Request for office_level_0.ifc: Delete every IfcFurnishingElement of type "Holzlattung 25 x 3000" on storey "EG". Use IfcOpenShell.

First a look at what the model holds.

```python
import ifcopenshell
import ifcopenshell.util.element

model = ifcopenshell.open("office_level_0.ifc")
print(model.schema)
storey = next(s for s in model.by_type("IfcBuildingStorey") if s.Name == "EG")
furniture = [e for e in ifcopenshell.util.element.get_decomposition(storey) if e.is_a("IfcFurnishingElement")]
seen = {}
for e in furniture:
    element_type = ifcopenshell.util.element.get_type(e)
    name = element_type.Name if element_type not in (None, e) else None
    seen[name] = seen.get(name, 0) + 1
for name, count in sorted(seen.items(), key=str):
    print(count, "x", name)
```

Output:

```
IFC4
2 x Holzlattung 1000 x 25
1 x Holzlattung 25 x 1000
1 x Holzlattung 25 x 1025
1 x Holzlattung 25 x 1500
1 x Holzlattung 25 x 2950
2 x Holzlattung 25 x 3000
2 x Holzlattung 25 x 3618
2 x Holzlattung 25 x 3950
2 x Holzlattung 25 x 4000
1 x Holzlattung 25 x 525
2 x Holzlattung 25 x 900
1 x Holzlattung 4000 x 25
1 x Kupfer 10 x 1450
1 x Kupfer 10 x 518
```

```python
import ifcopenshell
import ifcopenshell.api.root
import ifcopenshell.util.element

model = ifcopenshell.open("office_level_0.ifc")

storey = next(s for s in model.by_type("IfcBuildingStorey") if s.Name == "EG")
furniture = [e for e in ifcopenshell.util.element.get_decomposition(storey) if e.is_a("IfcFurnishingElement")]
targets = [e for e in furniture if (t := ifcopenshell.util.element.get_type(e)) not in (None, e) and t.Name == "Holzlattung 25 x 3000"]

for e in targets:
    ifcopenshell.api.root.remove_product(model, product=e)
print(len(targets), "removed")

model.write("office_level_0_v2.ifc")
```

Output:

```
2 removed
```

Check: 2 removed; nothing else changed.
